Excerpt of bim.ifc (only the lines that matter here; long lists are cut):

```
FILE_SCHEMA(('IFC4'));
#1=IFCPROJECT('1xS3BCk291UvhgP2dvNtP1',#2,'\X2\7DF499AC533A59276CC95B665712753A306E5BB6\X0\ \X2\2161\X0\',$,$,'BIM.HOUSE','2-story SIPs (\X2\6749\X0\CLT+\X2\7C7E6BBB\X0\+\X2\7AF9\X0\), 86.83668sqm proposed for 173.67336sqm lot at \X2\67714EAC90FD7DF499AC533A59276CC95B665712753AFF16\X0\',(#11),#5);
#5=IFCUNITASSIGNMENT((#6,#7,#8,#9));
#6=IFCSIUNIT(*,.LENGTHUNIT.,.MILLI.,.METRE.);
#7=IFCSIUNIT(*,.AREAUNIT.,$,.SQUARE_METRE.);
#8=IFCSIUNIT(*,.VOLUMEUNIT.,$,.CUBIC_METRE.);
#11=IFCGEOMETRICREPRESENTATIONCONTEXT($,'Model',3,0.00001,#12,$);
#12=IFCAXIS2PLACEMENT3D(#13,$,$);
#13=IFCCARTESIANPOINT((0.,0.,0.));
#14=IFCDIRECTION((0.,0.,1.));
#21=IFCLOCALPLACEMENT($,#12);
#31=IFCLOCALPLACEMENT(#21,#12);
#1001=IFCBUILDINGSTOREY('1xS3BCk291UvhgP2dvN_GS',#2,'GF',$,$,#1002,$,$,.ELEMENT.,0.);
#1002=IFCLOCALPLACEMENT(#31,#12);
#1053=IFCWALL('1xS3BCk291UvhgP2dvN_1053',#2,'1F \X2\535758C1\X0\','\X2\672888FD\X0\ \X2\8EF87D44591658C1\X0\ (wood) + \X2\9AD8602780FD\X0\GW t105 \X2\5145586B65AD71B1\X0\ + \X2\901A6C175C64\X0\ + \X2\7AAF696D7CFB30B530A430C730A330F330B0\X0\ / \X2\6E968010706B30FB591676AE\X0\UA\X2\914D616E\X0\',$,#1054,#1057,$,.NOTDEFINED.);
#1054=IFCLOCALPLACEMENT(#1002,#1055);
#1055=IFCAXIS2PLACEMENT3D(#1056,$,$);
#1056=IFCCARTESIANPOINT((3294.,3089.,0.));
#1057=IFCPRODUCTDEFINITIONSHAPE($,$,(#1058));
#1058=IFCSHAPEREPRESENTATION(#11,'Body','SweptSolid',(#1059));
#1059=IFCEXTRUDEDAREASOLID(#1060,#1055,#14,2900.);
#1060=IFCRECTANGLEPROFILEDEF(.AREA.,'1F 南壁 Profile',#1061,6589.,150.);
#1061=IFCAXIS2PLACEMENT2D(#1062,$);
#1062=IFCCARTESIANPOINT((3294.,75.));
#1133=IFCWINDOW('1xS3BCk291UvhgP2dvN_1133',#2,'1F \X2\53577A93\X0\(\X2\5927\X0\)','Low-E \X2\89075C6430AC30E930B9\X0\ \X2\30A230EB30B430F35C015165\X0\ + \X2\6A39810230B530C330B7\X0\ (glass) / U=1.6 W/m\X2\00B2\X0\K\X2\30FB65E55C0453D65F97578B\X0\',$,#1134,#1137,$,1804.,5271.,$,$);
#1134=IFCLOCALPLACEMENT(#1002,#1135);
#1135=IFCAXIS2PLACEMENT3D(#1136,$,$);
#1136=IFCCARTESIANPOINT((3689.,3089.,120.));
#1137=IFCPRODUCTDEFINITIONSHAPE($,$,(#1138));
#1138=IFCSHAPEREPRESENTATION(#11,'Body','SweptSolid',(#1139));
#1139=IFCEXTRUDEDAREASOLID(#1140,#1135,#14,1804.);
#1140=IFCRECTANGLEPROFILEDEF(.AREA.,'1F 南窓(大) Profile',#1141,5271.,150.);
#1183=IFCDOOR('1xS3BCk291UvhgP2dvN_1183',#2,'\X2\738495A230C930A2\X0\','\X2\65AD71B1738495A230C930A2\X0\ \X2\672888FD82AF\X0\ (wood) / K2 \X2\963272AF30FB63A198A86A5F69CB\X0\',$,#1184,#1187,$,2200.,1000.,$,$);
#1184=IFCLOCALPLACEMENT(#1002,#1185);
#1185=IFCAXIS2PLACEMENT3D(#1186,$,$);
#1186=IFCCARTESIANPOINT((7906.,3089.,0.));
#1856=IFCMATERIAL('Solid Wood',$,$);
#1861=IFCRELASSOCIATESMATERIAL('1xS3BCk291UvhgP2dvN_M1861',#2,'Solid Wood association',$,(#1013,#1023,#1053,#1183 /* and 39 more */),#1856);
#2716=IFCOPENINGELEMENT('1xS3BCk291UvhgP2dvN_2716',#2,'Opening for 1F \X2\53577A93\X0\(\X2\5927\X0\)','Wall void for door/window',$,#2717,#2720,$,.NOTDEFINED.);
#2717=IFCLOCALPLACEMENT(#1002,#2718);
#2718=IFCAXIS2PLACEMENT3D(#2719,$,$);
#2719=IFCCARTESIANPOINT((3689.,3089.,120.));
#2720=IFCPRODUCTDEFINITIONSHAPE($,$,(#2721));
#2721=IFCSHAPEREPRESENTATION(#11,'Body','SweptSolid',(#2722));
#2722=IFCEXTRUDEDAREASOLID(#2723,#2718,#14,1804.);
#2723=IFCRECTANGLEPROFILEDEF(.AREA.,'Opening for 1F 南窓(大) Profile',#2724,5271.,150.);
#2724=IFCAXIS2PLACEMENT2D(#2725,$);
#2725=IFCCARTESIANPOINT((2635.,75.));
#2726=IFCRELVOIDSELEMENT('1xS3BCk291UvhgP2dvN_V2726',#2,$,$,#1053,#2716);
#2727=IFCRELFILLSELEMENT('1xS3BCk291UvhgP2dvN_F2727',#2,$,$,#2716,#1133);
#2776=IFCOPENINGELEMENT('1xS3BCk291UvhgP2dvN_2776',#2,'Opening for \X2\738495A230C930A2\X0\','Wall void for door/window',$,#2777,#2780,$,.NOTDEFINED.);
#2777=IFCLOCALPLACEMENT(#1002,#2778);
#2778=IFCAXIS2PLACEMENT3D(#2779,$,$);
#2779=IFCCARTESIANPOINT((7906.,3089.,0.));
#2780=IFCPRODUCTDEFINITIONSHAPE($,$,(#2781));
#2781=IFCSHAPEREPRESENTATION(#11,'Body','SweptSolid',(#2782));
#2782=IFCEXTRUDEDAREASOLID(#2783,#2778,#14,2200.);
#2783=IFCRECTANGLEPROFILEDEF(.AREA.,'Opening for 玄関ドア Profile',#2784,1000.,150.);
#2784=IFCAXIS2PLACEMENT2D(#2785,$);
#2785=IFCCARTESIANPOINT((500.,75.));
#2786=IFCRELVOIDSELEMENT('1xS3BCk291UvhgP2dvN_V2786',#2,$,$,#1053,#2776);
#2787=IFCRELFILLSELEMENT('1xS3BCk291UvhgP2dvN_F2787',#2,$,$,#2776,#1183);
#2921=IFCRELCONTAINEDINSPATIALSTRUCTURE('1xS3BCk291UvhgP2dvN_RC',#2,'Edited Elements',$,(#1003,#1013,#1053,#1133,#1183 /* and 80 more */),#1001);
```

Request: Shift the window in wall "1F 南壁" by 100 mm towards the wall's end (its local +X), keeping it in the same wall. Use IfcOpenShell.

```python
import ifcopenshell
import ifcopenshell.api.geometry
import ifcopenshell.util.placement

model = ifcopenshell.open("bim.ifc")

window = model.by_guid("1xS3BCk291UvhgP2dvN_1133")
opening = window.FillsVoids[0].RelatingOpeningElement
wall = opening.VoidsElements[0].RelatingBuildingElement

wall_matrix = ifcopenshell.util.placement.get_local_placement(wall.ObjectPlacement)
shift = wall_matrix[:3, 0] * 100.0
before = ifcopenshell.util.placement.get_local_placement(window.ObjectPlacement)[:3, 3].copy()

# The window is not placed relative to its opening, so move both.
for product in (opening, window):
    matrix = ifcopenshell.util.placement.get_local_placement(product.ObjectPlacement)
    matrix[:3, 3] += shift
    ifcopenshell.api.geometry.edit_object_placement(model, product=product, matrix=matrix, is_si=False)

after = ifcopenshell.util.placement.get_local_placement(window.ObjectPlacement)[:3, 3]
print("window moved by", (after - before).round(3) + 0.0)

model.write("bim_updated.ifc")
```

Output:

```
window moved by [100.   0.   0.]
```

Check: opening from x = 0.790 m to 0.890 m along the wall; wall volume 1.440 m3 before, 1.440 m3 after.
